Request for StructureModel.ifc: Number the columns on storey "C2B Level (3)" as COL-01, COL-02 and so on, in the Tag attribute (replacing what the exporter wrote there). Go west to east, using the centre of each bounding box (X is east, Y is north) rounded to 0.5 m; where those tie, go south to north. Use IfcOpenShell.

First a look at what the model holds.

```python
import ifcopenshell
import ifcopenshell.util.element
import ifcopenshell.util.placement

model = ifcopenshell.open("StructureModel.ifc")
print(model.schema)
storey = next(s for s in model.by_type("IfcBuildingStorey") if s.Name == "C2B Level (3)")
columns = [e for e in ifcopenshell.util.element.get_decomposition(storey) if e.is_a("IfcColumn")]
for e in sorted(columns, key=lambda e: e.id()):
    origin = ifcopenshell.util.placement.get_local_placement(e.ObjectPlacement)[:3, 3]
    print(e.id(), e.Tag, e.Name, origin.round(2) + 0.0, sep=" | ")
```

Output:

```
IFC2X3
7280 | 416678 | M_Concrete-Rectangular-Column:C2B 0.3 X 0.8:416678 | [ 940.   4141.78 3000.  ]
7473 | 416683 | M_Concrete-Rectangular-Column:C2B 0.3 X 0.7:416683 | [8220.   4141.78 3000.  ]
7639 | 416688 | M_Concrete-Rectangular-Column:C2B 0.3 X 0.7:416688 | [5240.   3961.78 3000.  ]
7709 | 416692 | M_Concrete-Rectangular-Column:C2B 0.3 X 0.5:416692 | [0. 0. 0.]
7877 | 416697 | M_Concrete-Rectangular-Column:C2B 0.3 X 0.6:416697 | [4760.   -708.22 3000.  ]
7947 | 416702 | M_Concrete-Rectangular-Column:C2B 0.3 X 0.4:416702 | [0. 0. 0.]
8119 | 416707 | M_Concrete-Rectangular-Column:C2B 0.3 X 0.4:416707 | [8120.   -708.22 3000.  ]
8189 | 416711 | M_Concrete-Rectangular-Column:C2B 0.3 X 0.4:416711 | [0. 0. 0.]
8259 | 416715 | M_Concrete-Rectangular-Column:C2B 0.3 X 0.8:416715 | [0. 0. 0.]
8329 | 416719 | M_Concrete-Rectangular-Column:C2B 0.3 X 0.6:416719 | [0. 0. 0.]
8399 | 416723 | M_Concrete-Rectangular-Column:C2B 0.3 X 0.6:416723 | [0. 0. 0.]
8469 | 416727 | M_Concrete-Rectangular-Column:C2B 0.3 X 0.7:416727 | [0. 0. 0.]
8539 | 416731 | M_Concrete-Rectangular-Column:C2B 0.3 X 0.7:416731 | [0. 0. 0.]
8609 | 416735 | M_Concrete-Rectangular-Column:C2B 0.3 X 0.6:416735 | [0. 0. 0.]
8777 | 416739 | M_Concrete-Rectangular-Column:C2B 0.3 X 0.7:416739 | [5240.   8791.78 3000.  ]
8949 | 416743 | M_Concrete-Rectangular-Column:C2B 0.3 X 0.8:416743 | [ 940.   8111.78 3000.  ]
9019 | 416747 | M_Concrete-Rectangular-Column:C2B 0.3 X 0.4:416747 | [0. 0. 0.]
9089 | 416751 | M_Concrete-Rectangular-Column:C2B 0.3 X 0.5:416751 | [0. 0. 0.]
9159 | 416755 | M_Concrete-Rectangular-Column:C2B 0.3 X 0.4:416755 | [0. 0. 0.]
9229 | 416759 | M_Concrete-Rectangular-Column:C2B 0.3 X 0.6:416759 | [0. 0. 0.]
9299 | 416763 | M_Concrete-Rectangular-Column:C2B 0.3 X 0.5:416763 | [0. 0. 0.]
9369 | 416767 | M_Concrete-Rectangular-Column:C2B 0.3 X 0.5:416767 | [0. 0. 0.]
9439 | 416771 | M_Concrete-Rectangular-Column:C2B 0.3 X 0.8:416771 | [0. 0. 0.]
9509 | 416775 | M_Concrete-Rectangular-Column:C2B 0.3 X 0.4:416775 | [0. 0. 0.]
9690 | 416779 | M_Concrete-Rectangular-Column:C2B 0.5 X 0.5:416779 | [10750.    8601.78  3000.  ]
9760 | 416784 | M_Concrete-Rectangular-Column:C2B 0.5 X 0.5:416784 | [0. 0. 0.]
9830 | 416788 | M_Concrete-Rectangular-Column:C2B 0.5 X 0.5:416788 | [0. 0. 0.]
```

```python
import ifcopenshell
import ifcopenshell.geom
import ifcopenshell.util.element
import ifcopenshell.util.shape

model = ifcopenshell.open("StructureModel.ifc")
settings = ifcopenshell.geom.settings()
settings.set("use-world-coords", True)


def centre(element):
    shape = ifcopenshell.geom.create_shape(settings, element)
    return ifcopenshell.util.shape.get_bbox_centroid(shape.geometry)


storey = next(s for s in model.by_type("IfcBuildingStorey") if s.Name == "C2B Level (3)")
columns = [e for e in ifcopenshell.util.element.get_decomposition(storey) if e.is_a("IfcColumn")]

# Insertion points can sit at a corner or the storey origin, so sort by the geometry (in metres).
centres = {e: centre(e) for e in columns}
columns.sort(key=lambda e: (round(centres[e][0] / 0.5), centres[e][1]))

for i, e in enumerate(columns, start=1):
    number = f"COL-{i:02d}"
    e.Tag = number
    print(e.id(), number)

model.write("StructureModel_v2.ifc")
```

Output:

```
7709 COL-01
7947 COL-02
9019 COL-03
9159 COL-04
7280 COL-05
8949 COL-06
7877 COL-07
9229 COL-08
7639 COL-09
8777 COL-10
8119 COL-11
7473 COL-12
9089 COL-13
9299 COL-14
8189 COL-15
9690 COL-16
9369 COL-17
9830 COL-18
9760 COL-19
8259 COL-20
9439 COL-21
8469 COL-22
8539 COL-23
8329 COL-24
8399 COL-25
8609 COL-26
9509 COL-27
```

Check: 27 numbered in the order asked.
